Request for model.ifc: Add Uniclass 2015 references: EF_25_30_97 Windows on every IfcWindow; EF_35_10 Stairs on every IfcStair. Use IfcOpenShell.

First a look at what the model holds.

```python
import ifcopenshell

model = ifcopenshell.open("model.ifc")
print(model.schema)
print("classifications:", [c.Name for c in model.by_type("IfcClassification")])
for ifc_class in ("IfcDoor", "IfcRoof", "IfcStair", "IfcWall", "IfcWindow"):
    print(ifc_class, len(model.by_type(ifc_class)))
```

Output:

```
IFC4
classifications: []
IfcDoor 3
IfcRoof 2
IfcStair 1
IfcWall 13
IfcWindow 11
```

```python
import ifcopenshell
import ifcopenshell.api.classification

model = ifcopenshell.open("model.ifc")

system = ifcopenshell.api.classification.add_classification(model, classification="Uniclass 2015")

codes = {
    "IfcWindow": ("EF_25_30_97", "Windows"),
    "IfcStair": ("EF_35_10", "Stairs"),
}
for ifc_class, (code, name) in codes.items():
    products = model.by_type(ifc_class)
    ifcopenshell.api.classification.add_reference(
        model, products=products, classification=system, identification=code, name=name
    )
    print(code, len(products))

model.write("model_edited.ifc")
```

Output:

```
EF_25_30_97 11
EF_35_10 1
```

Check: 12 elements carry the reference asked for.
